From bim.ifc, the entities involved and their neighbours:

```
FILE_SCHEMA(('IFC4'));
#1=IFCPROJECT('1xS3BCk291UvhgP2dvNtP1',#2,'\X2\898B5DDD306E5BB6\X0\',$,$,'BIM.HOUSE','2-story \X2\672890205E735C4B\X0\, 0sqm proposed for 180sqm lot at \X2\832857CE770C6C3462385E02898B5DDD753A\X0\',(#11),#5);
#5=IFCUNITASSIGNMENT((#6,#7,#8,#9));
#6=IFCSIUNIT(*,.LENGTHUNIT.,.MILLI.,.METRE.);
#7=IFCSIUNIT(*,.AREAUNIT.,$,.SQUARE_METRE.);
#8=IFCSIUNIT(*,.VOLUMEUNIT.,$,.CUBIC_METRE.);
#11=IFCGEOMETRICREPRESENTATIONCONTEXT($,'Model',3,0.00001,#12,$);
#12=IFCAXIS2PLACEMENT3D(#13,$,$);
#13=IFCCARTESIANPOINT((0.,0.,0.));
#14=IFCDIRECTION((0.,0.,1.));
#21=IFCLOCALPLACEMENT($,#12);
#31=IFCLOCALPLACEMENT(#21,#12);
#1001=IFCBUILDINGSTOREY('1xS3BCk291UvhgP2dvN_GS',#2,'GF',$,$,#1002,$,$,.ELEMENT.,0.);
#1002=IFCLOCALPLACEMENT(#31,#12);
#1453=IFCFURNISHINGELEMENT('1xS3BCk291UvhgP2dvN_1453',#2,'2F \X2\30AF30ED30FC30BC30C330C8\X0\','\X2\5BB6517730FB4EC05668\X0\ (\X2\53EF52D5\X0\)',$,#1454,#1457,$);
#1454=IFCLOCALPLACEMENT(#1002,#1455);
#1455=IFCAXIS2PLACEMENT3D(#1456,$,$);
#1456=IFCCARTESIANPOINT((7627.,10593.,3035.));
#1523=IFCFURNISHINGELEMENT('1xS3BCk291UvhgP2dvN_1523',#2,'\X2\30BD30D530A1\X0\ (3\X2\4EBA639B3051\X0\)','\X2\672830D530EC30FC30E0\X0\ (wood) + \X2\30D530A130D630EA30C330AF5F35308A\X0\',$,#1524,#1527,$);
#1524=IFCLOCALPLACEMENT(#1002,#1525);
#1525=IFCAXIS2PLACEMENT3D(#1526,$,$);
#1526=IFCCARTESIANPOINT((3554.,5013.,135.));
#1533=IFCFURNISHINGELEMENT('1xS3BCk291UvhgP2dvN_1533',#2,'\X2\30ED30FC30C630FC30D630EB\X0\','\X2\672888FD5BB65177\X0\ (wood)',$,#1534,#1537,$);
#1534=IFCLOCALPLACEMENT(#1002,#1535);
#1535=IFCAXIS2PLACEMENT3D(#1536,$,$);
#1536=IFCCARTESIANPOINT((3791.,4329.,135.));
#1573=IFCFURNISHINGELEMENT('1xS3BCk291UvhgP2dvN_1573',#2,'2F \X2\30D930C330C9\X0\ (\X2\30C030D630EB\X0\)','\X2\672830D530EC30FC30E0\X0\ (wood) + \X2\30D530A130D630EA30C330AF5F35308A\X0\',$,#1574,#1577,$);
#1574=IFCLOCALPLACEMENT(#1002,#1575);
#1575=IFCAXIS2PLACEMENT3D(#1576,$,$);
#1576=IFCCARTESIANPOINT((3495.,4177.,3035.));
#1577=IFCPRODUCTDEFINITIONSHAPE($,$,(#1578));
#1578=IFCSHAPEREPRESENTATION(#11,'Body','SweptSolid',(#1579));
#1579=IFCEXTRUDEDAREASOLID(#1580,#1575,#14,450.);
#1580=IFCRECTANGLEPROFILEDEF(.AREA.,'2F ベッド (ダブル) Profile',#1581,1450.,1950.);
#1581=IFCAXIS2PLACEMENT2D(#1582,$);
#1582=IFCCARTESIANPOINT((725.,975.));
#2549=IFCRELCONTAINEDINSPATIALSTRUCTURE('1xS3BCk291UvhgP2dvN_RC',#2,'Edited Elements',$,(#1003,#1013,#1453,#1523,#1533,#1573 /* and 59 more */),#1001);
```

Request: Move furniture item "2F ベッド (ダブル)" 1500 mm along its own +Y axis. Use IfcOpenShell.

```python
import ifcopenshell
import ifcopenshell.api.geometry
import ifcopenshell.util.placement
import ifcopenshell.util.unit

model = ifcopenshell.open("bim.ifc")
unit_scale = ifcopenshell.util.unit.calculate_unit_scale(model)

item = model.by_id(1573)
matrix = ifcopenshell.util.placement.get_local_placement(item.ObjectPlacement)
matrix[:3, 3] += matrix[:3, 1] * 1.5 / unit_scale
ifcopenshell.api.geometry.edit_object_placement(model, product=item, matrix=matrix, is_si=False)

print(ifcopenshell.util.placement.get_local_placement(item.ObjectPlacement).round(3) + 0.0)

model.write("bim_edited.ifc")
```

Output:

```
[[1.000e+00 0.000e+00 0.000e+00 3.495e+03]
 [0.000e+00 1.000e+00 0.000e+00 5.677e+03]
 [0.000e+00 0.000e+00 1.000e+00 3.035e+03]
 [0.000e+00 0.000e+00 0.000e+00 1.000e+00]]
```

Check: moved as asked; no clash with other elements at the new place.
